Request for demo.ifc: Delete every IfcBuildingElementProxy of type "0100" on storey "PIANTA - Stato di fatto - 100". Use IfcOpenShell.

First a look at what the model holds.

```python
import ifcopenshell
import ifcopenshell.util.element

model = ifcopenshell.open("demo.ifc")
print(model.schema)
storey = next(s for s in model.by_type("IfcBuildingStorey") if s.Name == "PIANTA - Stato di fatto - 100")
proxies = [e for e in ifcopenshell.util.element.get_decomposition(storey) if e.is_a("IfcBuildingElementProxy")]
seen = {}
for e in proxies:
    element_type = ifcopenshell.util.element.get_type(e)
    name = element_type.Name if element_type not in (None, e) else None
    seen[name] = seen.get(name, 0) + 1
for name, count in sorted(seen.items(), key=str):
    print(count, "x", name)
```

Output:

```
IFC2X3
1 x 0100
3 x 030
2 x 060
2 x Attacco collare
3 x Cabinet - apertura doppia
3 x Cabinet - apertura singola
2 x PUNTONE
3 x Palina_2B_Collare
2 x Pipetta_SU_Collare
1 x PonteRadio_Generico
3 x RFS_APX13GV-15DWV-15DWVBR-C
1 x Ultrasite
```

```python
import ifcopenshell
import ifcopenshell.api.root
import ifcopenshell.util.element

model = ifcopenshell.open("demo.ifc")

storey = next(s for s in model.by_type("IfcBuildingStorey") if s.Name == "PIANTA - Stato di fatto - 100")
proxies = [e for e in ifcopenshell.util.element.get_decomposition(storey) if e.is_a("IfcBuildingElementProxy")]
targets = [e for e in proxies if (t := ifcopenshell.util.element.get_type(e)) not in (None, e) and t.Name == "0100"]

for e in targets:
    ifcopenshell.api.root.remove_product(model, product=e)
print(len(targets), "removed")

model.write("demo_edited.ifc")
```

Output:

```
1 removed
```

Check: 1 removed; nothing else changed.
